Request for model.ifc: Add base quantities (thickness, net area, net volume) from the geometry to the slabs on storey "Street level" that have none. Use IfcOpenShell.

First a look at what the model holds.

```python
import ifcopenshell
import ifcopenshell.util.element
import ifcopenshell.util.unit

model = ifcopenshell.open("model.ifc")
print(model.schema)
for unit_type in ("LENGTHUNIT", "AREAUNIT", "VOLUMEUNIT"):
    print(unit_type, ifcopenshell.util.unit.calculate_unit_scale(model, unit_type))
storey = next(s for s in model.by_type("IfcBuildingStorey") if s.Name == "Street level")
slabs = [e for e in ifcopenshell.util.element.get_decomposition(storey) if e.is_a("IfcSlab")]
for e in sorted(slabs, key=lambda e: e.id()):
    print(e.id(), e.is_a(), e.Name, list(ifcopenshell.util.element.get_psets(e, qtos_only=True)), sep=" | ")
```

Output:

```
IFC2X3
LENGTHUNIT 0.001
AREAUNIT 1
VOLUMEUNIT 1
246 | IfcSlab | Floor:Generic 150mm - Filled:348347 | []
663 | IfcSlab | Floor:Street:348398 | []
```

```python
import ifcopenshell
import ifcopenshell.api.pset
import ifcopenshell.geom
import ifcopenshell.util.element
import ifcopenshell.util.shape
import ifcopenshell.util.unit

model = ifcopenshell.open("model.ifc")
unit_scale = ifcopenshell.util.unit.calculate_unit_scale(model)
area_scale = ifcopenshell.util.unit.calculate_unit_scale(model, "AREAUNIT")
volume_scale = ifcopenshell.util.unit.calculate_unit_scale(model, "VOLUMEUNIT")
settings = ifcopenshell.geom.settings()

storey = next(s for s in model.by_type("IfcBuildingStorey") if s.Name == "Street level")
slabs = [e for e in ifcopenshell.util.element.get_decomposition(storey) if e.is_a("IfcSlab")]

for e in sorted(slabs, key=lambda e: e.id()):
    if ifcopenshell.util.element.get_psets(e, qtos_only=True, should_inherit=False):
        continue
    # Geometry comes back in metres, in the element's own axes.
    shape = ifcopenshell.geom.create_shape(settings, e)
    values = {
        "Width": ifcopenshell.util.shape.get_z(shape.geometry) / unit_scale,
        "NetArea": ifcopenshell.util.shape.get_footprint_area(shape.geometry) / area_scale,
        "NetVolume": ifcopenshell.util.shape.get_volume(shape.geometry) / volume_scale,
    }
    qto = ifcopenshell.api.pset.add_qto(model, product=e, name="BaseQuantities")
    ifcopenshell.api.pset.edit_qto(model, qto=qto, properties=values)
    print(e.id(), {k: round(v, 3) for k, v in values.items()})

model.write("model_updated.ifc")
```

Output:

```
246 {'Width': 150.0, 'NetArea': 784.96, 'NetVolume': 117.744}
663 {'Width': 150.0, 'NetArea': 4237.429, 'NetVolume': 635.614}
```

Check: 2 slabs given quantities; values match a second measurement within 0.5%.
